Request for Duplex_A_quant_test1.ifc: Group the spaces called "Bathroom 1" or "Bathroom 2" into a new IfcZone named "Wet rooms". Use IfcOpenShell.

First a look at what the model holds.

```python
import ifcopenshell

model = ifcopenshell.open("Duplex_A_quant_test1.ifc")
print(model.schema)
seen = {}
for space in model.by_type("IfcSpace"):
    seen[space.LongName] = seen.get(space.LongName, 0) + 1
for name, count in sorted(seen.items(), key=str):
    print(count, "x", name)
print("zones:", [z.Name for z in model.by_type("IfcZone")][:20])
```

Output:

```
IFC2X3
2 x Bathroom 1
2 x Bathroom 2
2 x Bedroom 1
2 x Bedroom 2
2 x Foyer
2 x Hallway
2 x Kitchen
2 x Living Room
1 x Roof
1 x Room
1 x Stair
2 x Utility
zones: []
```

```python
import ifcopenshell
import ifcopenshell.api.group
import ifcopenshell.api.root

model = ifcopenshell.open("Duplex_A_quant_test1.ifc")

names = {"Bathroom 1", "Bathroom 2"}
spaces = [s for s in model.by_type("IfcSpace") if s.LongName in names]

zone = ifcopenshell.api.root.create_entity(model, ifc_class="IfcZone", name="Wet rooms")
ifcopenshell.api.group.assign_group(model, products=spaces, group=zone)
print(len(spaces), "spaces in", zone.Name)

model.write("Duplex_A_quant_test1_rev.ifc")
```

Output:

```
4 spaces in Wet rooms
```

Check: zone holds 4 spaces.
